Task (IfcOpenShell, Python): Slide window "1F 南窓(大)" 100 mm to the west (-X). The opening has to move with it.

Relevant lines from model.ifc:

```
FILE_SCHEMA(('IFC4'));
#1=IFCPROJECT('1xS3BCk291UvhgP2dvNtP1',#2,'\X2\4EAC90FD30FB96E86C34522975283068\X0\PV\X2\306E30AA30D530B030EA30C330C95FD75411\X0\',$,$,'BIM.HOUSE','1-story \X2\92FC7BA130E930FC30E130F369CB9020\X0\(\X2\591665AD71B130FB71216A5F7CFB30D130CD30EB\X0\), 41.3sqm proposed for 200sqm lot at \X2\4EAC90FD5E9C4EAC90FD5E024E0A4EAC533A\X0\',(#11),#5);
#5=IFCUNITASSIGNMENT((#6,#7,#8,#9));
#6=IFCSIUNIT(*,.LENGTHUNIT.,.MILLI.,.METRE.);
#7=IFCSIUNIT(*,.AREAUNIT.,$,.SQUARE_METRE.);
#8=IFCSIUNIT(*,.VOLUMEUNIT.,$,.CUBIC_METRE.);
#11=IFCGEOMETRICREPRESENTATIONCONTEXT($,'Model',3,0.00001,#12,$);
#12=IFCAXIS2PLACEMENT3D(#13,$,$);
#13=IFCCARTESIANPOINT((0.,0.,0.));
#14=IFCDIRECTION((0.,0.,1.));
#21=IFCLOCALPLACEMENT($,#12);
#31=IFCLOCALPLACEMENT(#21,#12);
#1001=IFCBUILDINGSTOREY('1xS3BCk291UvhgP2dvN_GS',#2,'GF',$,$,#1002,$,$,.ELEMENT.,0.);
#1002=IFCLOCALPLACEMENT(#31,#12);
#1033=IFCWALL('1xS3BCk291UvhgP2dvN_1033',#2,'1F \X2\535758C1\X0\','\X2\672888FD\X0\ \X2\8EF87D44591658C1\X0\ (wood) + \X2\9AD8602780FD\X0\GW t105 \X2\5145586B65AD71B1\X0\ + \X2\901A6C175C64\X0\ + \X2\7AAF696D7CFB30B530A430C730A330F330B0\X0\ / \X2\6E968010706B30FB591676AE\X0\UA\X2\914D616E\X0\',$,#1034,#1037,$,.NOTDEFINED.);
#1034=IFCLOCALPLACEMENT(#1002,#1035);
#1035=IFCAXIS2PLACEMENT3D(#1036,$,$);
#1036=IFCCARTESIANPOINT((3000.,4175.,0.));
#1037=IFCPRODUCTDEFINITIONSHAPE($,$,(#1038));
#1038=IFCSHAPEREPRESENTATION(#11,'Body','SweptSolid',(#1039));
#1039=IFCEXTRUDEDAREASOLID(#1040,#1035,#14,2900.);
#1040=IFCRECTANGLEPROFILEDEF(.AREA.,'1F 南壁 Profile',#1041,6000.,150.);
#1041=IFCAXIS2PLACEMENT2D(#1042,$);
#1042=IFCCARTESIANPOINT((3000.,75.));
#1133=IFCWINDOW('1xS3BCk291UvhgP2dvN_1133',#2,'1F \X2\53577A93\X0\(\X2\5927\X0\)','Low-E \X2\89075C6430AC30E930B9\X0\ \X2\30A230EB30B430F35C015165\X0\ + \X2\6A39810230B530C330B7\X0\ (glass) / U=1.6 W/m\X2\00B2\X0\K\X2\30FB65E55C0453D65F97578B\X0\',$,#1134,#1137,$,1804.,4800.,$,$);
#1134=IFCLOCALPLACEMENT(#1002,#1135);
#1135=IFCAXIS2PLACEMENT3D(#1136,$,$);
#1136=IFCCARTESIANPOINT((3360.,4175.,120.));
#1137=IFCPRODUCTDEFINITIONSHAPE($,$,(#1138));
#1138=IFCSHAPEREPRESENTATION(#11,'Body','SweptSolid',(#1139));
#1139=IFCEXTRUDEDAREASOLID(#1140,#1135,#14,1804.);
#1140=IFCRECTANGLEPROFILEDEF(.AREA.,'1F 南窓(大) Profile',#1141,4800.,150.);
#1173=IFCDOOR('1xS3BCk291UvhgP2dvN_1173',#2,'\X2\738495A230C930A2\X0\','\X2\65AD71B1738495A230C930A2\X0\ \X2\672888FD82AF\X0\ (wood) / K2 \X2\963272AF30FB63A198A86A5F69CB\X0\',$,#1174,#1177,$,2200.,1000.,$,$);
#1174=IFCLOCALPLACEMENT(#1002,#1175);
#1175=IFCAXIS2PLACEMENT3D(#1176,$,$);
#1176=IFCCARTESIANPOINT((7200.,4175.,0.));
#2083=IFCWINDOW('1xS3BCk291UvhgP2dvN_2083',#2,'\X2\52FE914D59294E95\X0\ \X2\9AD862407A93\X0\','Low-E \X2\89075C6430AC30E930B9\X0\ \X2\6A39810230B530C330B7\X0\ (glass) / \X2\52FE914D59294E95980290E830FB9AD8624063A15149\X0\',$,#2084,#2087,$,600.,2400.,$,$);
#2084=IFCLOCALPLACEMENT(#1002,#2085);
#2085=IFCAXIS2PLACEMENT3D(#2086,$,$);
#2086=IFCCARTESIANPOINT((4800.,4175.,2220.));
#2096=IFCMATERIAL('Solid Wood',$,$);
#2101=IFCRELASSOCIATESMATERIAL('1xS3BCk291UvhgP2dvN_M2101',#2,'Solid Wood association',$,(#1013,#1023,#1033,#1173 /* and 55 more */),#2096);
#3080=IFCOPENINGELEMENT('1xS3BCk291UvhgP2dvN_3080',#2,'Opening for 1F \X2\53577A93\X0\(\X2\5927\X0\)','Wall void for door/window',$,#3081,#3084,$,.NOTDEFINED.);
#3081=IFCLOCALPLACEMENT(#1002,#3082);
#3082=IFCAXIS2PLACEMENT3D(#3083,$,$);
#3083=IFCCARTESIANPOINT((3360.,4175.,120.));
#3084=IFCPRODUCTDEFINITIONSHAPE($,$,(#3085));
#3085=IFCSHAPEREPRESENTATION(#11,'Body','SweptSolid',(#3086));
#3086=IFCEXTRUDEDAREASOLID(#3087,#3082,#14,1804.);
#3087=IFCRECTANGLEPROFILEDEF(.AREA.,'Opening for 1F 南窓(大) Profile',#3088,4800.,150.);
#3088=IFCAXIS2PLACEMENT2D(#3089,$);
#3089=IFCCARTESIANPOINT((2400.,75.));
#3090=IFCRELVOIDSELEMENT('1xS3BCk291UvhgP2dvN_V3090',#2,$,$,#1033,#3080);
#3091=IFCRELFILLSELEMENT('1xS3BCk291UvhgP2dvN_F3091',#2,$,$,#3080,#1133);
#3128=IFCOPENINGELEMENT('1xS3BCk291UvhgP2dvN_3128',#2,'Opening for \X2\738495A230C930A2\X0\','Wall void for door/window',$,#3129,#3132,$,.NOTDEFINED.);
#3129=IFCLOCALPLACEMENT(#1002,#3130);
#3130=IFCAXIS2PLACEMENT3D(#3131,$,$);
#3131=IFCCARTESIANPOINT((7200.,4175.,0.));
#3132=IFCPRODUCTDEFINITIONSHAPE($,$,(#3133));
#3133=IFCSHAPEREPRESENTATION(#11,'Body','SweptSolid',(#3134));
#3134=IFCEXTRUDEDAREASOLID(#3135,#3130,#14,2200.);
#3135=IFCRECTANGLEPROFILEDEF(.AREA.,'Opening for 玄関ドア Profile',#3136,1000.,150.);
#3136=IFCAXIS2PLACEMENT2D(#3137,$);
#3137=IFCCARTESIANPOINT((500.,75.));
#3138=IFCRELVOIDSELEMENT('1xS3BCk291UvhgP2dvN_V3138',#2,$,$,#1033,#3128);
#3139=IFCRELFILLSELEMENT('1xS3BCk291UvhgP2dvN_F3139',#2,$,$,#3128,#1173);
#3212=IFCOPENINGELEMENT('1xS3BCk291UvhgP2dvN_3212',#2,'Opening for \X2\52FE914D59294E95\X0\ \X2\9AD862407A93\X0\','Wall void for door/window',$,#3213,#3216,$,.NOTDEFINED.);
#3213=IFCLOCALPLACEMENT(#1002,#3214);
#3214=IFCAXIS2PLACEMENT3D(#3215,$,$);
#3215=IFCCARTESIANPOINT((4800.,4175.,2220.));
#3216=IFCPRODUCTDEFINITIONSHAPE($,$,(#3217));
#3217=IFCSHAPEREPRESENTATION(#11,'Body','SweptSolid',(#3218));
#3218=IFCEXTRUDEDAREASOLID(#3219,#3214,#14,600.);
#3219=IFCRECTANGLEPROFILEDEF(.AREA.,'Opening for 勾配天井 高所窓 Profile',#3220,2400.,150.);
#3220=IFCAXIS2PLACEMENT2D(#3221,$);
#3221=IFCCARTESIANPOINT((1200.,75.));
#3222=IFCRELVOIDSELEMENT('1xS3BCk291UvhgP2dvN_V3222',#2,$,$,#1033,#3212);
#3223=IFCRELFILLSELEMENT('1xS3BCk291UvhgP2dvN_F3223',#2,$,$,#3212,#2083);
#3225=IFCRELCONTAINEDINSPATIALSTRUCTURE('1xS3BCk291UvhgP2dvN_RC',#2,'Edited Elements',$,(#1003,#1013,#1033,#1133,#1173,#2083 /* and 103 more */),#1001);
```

```python
import ifcopenshell
import ifcopenshell.api.geometry
import ifcopenshell.util.placement

model = ifcopenshell.open("model.ifc")

window = model.by_guid("1xS3BCk291UvhgP2dvN_1133")
opening = window.FillsVoids[0].RelatingOpeningElement
wall = opening.VoidsElements[0].RelatingBuildingElement

wall_matrix = ifcopenshell.util.placement.get_local_placement(wall.ObjectPlacement)
shift = wall_matrix[:3, 0] * -100.0
before = ifcopenshell.util.placement.get_local_placement(window.ObjectPlacement)[:3, 3].copy()

# The window is not placed relative to its opening, so move both.
for product in (opening, window):
    matrix = ifcopenshell.util.placement.get_local_placement(product.ObjectPlacement)
    matrix[:3, 3] += shift
    ifcopenshell.api.geometry.edit_object_placement(model, product=product, matrix=matrix, is_si=False)

after = ifcopenshell.util.placement.get_local_placement(window.ObjectPlacement)[:3, 3]
print("window moved by", (after - before).round(3) + 0.0)

model.write("model_updated.ifc")
```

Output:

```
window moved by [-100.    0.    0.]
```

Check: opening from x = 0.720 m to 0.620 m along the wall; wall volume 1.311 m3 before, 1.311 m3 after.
